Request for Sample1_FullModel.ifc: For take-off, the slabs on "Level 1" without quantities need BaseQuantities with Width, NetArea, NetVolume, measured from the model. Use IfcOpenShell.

First a look at what the model holds.

```python
import ifcopenshell
import ifcopenshell.util.element
import ifcopenshell.util.unit

model = ifcopenshell.open("Sample1_FullModel.ifc")
print(model.schema)
for unit_type in ("LENGTHUNIT", "AREAUNIT", "VOLUMEUNIT"):
    print(unit_type, ifcopenshell.util.unit.calculate_unit_scale(model, unit_type))
storey = next(s for s in model.by_type("IfcBuildingStorey") if s.Name == "Level 1")
slabs = [e for e in ifcopenshell.util.element.get_decomposition(storey) if e.is_a("IfcSlab")]
for e in sorted(slabs, key=lambda e: e.id()):
    print(e.id(), e.is_a(), e.Name, list(ifcopenshell.util.element.get_psets(e, qtos_only=True)), sep=" | ")
```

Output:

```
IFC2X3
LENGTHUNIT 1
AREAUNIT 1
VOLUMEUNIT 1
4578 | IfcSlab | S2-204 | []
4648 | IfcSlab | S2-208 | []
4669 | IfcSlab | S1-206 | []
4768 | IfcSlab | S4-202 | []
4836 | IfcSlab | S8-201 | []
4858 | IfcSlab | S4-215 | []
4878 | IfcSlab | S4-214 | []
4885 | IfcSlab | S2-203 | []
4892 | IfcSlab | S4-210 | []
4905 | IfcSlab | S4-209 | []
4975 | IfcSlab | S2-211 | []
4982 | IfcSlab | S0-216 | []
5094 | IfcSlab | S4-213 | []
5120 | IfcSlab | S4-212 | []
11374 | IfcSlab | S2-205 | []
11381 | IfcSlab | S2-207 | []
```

```python
import ifcopenshell
import ifcopenshell.api.pset
import ifcopenshell.geom
import ifcopenshell.util.element
import ifcopenshell.util.shape
import ifcopenshell.util.unit

model = ifcopenshell.open("Sample1_FullModel.ifc")
unit_scale = ifcopenshell.util.unit.calculate_unit_scale(model)
area_scale = ifcopenshell.util.unit.calculate_unit_scale(model, "AREAUNIT")
volume_scale = ifcopenshell.util.unit.calculate_unit_scale(model, "VOLUMEUNIT")
settings = ifcopenshell.geom.settings()

storey = next(s for s in model.by_type("IfcBuildingStorey") if s.Name == "Level 1")
slabs = [e for e in ifcopenshell.util.element.get_decomposition(storey) if e.is_a("IfcSlab")]

for e in sorted(slabs, key=lambda e: e.id()):
    if ifcopenshell.util.element.get_psets(e, qtos_only=True, should_inherit=False):
        continue
    # Geometry comes back in metres, in the element's own axes.
    shape = ifcopenshell.geom.create_shape(settings, e)
    values = {
        "Width": ifcopenshell.util.shape.get_z(shape.geometry) / unit_scale,
        "NetArea": ifcopenshell.util.shape.get_footprint_area(shape.geometry) / area_scale,
        "NetVolume": ifcopenshell.util.shape.get_volume(shape.geometry) / volume_scale,
    }
    qto = ifcopenshell.api.pset.add_qto(model, product=e, name="BaseQuantities")
    ifcopenshell.api.pset.edit_qto(model, qto=qto, properties=values)
    print(e.id(), {k: round(v, 3) for k, v in values.items()})

model.write("Sample1_FullModel-out.ifc")
```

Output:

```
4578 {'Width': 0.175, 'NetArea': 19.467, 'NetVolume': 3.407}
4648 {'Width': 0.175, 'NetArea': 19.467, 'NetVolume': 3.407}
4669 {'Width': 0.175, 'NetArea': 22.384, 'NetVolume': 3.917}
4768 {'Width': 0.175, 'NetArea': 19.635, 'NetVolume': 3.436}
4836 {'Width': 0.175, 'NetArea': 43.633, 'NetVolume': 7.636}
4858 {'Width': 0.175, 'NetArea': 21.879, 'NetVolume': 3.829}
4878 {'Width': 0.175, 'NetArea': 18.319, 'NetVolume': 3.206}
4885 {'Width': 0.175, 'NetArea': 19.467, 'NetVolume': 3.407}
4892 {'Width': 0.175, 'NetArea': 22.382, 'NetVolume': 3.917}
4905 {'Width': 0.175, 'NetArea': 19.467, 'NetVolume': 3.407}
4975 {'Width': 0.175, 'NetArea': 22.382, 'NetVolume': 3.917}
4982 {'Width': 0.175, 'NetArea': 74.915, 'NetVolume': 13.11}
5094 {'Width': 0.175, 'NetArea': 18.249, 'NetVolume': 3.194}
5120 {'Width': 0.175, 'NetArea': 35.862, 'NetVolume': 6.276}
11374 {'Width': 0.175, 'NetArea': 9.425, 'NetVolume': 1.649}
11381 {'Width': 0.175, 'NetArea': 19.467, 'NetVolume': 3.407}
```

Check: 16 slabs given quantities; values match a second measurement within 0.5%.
